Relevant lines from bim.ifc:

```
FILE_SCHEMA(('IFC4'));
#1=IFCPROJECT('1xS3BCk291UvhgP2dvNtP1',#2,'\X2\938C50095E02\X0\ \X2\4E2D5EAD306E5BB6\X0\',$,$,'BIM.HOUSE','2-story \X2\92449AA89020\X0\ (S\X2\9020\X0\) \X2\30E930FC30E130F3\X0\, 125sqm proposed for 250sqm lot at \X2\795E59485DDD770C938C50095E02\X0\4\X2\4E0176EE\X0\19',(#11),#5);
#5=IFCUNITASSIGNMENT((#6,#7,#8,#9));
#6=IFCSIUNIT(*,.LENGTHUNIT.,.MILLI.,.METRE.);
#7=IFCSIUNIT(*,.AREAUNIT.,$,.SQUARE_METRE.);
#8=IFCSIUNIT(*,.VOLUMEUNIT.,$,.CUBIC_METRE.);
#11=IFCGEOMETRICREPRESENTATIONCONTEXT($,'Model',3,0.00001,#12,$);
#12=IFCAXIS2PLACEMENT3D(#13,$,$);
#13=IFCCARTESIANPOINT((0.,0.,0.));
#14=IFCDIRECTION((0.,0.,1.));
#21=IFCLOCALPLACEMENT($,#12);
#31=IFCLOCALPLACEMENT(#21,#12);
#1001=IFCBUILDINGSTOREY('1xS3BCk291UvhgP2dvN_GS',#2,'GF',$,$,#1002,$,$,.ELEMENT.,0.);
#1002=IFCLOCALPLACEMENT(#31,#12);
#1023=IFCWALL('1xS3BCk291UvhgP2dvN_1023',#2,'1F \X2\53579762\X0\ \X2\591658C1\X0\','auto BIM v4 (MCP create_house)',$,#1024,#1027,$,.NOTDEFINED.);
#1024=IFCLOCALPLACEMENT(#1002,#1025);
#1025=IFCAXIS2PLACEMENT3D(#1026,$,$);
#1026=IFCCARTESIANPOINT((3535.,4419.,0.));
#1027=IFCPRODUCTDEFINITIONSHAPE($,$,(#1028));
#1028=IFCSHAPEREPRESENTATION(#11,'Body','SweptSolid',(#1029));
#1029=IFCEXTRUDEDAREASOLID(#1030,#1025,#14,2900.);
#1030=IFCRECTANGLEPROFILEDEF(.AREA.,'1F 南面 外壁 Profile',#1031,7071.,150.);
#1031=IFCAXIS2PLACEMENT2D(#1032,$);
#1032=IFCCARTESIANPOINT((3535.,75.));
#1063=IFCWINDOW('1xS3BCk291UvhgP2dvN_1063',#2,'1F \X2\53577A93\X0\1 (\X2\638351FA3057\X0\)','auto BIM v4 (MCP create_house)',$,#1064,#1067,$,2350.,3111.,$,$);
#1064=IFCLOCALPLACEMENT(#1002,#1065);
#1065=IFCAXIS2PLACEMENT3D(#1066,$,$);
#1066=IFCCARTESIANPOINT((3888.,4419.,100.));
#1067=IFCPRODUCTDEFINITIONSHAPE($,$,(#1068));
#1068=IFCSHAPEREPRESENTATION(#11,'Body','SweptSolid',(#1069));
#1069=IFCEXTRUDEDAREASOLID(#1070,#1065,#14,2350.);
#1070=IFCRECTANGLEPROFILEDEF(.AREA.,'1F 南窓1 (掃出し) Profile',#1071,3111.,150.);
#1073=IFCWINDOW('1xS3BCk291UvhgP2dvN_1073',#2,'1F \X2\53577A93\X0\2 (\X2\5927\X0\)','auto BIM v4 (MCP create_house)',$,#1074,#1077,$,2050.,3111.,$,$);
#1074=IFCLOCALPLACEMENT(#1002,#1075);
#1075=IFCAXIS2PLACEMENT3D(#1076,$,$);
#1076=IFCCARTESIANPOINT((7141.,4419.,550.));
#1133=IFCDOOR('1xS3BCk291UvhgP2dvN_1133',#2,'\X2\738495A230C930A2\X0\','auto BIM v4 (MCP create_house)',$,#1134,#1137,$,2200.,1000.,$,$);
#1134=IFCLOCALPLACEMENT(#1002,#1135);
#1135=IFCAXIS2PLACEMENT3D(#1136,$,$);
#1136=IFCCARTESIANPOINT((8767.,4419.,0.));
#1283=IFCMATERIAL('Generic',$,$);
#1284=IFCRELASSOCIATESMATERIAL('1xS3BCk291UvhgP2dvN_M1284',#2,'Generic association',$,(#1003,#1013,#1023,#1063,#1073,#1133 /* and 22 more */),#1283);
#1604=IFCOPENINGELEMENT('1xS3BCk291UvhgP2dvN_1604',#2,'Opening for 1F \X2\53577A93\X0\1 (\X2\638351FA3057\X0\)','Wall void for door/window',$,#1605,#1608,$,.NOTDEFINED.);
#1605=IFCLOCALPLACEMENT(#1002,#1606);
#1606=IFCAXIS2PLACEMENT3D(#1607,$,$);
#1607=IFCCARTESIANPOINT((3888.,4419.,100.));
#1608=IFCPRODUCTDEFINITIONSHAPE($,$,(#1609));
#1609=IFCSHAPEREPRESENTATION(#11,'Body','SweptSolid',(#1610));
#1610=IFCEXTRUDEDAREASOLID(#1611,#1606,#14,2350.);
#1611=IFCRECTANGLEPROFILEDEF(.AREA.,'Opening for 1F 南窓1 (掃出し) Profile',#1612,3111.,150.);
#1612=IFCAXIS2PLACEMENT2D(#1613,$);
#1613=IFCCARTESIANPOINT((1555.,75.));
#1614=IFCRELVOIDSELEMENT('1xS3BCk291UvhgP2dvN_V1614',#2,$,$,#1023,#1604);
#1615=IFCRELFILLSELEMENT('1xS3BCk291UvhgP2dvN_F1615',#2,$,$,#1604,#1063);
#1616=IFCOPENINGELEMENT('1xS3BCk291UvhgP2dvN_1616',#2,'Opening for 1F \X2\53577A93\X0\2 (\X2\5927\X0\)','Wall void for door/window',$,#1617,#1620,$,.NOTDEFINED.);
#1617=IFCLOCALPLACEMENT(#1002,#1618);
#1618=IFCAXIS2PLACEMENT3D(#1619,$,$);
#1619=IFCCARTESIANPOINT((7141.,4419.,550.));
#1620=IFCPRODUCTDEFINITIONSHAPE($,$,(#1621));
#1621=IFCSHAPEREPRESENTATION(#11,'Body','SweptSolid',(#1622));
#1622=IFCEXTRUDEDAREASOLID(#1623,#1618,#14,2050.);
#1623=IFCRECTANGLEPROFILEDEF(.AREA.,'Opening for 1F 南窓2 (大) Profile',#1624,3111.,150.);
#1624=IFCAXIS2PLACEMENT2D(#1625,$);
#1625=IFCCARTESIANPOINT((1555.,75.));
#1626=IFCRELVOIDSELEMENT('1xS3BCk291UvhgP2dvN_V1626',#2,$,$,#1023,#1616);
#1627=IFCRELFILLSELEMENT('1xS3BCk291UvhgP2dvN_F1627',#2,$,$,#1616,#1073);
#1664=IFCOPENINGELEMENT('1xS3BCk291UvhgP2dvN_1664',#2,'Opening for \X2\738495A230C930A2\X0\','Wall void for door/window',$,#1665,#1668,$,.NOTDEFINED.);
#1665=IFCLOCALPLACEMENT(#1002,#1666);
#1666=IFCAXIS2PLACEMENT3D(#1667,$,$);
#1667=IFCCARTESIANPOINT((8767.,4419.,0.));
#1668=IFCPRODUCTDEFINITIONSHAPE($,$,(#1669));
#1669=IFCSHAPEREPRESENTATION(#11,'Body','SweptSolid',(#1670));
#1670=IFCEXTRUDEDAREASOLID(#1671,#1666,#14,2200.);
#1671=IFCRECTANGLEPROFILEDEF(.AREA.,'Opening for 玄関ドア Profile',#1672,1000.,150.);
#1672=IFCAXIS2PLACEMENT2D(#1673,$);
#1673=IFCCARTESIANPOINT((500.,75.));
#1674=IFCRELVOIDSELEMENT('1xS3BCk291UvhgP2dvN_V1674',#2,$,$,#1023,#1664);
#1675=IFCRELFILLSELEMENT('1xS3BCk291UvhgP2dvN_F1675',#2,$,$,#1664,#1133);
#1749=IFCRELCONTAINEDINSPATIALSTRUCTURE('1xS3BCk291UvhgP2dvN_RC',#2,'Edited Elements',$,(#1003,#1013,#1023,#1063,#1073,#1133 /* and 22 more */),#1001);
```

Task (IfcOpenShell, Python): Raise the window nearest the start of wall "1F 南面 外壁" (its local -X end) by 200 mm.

```python
import numpy as np
import ifcopenshell
import ifcopenshell.api.geometry
import ifcopenshell.util.placement
import ifcopenshell.util.unit

model = ifcopenshell.open("bim.ifc")
unit_scale = ifcopenshell.util.unit.calculate_unit_scale(model)

window = model.by_id(1063)
opening = window.FillsVoids[0].RelatingOpeningElement
dz = 200.0

shift = np.array([0.0, 0.0, dz])
# The window is not placed relative to its opening, so move both.
for product in (opening, window):
    matrix = ifcopenshell.util.placement.get_local_placement(product.ObjectPlacement)
    matrix[:3, 3] += shift
    ifcopenshell.api.geometry.edit_object_placement(model, product=product, matrix=matrix, is_si=False)

print(f"moved by {dz * unit_scale:+.3f} m")

model.write("bim_edited.ifc")
```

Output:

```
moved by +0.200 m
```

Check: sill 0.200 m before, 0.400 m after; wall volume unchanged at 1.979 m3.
